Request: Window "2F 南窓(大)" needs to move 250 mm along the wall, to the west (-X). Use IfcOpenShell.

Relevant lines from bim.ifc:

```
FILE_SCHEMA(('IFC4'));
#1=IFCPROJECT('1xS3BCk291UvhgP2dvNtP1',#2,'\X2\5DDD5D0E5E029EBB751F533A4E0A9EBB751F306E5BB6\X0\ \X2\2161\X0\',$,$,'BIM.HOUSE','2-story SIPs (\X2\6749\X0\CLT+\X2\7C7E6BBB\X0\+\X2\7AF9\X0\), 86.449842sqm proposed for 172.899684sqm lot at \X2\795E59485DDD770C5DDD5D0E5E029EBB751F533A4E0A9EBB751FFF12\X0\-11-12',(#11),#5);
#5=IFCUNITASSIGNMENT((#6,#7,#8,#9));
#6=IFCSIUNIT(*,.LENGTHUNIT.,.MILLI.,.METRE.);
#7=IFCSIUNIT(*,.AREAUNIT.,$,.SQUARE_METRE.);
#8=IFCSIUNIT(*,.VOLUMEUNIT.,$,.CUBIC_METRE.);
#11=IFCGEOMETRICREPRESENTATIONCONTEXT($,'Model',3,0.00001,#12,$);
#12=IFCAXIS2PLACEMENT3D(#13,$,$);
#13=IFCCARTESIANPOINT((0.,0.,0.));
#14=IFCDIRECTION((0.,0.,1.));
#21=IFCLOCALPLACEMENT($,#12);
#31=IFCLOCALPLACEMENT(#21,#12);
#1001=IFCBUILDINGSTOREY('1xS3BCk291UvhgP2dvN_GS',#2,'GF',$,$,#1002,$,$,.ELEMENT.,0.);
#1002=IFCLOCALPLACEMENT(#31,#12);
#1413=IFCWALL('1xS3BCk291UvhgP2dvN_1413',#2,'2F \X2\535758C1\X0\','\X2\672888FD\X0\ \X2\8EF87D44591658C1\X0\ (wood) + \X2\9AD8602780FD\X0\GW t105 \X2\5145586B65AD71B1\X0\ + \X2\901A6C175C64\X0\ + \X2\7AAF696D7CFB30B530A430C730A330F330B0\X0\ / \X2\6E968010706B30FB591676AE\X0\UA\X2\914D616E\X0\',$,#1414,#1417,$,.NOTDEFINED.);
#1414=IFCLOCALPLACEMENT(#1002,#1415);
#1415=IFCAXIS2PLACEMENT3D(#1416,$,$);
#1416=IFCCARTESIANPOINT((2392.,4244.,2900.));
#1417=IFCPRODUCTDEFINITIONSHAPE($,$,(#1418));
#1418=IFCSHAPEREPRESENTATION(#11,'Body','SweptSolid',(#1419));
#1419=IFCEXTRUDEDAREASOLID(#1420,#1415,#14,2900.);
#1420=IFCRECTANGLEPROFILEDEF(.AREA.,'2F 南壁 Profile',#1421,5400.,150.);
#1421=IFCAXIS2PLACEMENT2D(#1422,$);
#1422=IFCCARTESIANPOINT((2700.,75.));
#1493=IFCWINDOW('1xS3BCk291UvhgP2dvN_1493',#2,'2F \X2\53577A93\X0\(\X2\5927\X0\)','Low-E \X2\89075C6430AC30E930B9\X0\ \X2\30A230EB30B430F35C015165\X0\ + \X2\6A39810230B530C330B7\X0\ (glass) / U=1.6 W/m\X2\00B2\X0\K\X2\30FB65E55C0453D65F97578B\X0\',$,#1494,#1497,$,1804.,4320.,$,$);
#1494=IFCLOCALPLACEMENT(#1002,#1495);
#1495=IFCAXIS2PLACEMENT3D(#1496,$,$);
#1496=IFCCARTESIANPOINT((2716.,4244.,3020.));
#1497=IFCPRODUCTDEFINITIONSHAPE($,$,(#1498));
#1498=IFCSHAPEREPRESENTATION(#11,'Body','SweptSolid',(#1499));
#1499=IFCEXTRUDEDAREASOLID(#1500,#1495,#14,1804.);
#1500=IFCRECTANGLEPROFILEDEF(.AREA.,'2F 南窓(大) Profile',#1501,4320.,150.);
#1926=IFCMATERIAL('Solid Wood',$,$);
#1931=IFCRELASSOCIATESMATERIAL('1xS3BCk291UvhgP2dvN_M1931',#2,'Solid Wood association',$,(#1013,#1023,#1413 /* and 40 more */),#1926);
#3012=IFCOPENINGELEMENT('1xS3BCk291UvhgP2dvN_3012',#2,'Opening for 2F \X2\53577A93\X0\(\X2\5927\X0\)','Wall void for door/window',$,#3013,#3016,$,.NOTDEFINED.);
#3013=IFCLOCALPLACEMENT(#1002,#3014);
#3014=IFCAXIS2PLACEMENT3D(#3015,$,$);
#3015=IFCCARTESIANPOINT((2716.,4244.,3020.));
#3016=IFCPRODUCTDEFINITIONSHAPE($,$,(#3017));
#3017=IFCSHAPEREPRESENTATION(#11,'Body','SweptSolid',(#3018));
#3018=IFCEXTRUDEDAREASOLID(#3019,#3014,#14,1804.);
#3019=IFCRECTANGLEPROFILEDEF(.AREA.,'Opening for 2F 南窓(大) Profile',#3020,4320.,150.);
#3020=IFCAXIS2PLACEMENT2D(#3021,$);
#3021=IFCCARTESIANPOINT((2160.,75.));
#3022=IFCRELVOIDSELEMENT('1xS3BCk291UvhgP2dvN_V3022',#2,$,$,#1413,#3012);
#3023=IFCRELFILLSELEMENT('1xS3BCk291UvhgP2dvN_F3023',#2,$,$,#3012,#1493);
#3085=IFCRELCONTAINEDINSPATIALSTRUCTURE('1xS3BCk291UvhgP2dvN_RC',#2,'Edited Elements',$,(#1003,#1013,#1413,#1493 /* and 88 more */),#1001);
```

```python
import ifcopenshell
import ifcopenshell.api.geometry
import ifcopenshell.util.placement
import ifcopenshell.util.unit

model = ifcopenshell.open("bim.ifc")
unit_scale = ifcopenshell.util.unit.calculate_unit_scale(model)

window = model.by_guid("1xS3BCk291UvhgP2dvN_1493")
opening = window.FillsVoids[0].RelatingOpeningElement
wall = opening.VoidsElements[0].RelatingBuildingElement

wall_matrix = ifcopenshell.util.placement.get_local_placement(wall.ObjectPlacement)
shift = wall_matrix[:3, 0] * -0.25 / unit_scale
before = ifcopenshell.util.placement.get_local_placement(window.ObjectPlacement)[:3, 3].copy()

# The window is not placed relative to its opening, so move both.
for product in (opening, window):
    matrix = ifcopenshell.util.placement.get_local_placement(product.ObjectPlacement)
    matrix[:3, 3] += shift
    ifcopenshell.api.geometry.edit_object_placement(model, product=product, matrix=matrix, is_si=False)

after = ifcopenshell.util.placement.get_local_placement(window.ObjectPlacement)[:3, 3]
print("window moved by", (after - before).round(3) + 0.0)

model.write("bim_rev.ifc")
```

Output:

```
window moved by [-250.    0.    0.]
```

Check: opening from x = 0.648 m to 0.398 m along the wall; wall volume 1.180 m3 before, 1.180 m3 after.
